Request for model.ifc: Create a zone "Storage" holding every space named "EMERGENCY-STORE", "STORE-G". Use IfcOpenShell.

First a look at what the model holds.

```python
import ifcopenshell

model = ifcopenshell.open("model.ifc")
print(model.schema)
seen = {}
for space in model.by_type("IfcSpace"):
    seen[space.Name] = seen.get(space.Name, 0) + 1
for name, count in sorted(seen.items(), key=str):
    print(count, "x", name)
print("zones:", [z.Name for z in model.by_type("IfcZone")][:20])
```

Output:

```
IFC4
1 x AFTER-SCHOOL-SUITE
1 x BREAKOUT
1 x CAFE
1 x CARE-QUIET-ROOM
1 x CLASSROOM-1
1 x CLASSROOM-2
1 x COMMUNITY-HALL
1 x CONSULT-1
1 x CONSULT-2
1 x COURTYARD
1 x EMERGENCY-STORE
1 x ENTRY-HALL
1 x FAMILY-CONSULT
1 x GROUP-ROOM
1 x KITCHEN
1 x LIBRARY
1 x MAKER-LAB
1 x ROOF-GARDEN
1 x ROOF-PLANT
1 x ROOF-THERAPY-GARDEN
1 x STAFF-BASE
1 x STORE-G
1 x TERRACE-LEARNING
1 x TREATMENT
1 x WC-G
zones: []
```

```python
import ifcopenshell
import ifcopenshell.api.group
import ifcopenshell.api.root

model = ifcopenshell.open("model.ifc")

names = {"EMERGENCY-STORE", "STORE-G"}
spaces = [s for s in model.by_type("IfcSpace") if s.Name in names]

zone = ifcopenshell.api.root.create_entity(model, ifc_class="IfcZone", name="Storage")
ifcopenshell.api.group.assign_group(model, products=spaces, group=zone)
print(len(spaces), "spaces in", zone.Name)

model.write("model_updated.ifc")
```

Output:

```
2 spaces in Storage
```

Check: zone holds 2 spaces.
